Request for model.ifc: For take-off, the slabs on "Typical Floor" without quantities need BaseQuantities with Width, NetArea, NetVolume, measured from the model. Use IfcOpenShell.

First a look at what the model holds.

```python
import ifcopenshell
import ifcopenshell.util.element
import ifcopenshell.util.unit

model = ifcopenshell.open("model.ifc")
print(model.schema)
for unit_type in ("LENGTHUNIT", "AREAUNIT", "VOLUMEUNIT"):
    print(unit_type, ifcopenshell.util.unit.calculate_unit_scale(model, unit_type))
storey = next(s for s in model.by_type("IfcBuildingStorey") if s.Name == "Typical Floor")
slabs = [e for e in ifcopenshell.util.element.get_decomposition(storey) if e.is_a("IfcSlab")]
for e in sorted(slabs, key=lambda e: e.id()):
    print(e.id(), e.is_a(), e.Name, list(ifcopenshell.util.element.get_psets(e, qtos_only=True)), sep=" | ")
```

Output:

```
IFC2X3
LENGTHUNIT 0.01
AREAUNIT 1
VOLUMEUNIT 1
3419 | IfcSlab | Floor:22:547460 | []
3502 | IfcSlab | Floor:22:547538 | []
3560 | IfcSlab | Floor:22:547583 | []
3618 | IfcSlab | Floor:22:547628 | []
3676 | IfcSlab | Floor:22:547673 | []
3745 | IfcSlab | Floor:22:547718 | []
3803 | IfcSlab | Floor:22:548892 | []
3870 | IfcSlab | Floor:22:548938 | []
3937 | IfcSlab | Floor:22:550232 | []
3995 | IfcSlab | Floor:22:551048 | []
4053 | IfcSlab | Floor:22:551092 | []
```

```python
import ifcopenshell
import ifcopenshell.api.pset
import ifcopenshell.geom
import ifcopenshell.util.element
import ifcopenshell.util.shape
import ifcopenshell.util.unit

model = ifcopenshell.open("model.ifc")
unit_scale = ifcopenshell.util.unit.calculate_unit_scale(model)
area_scale = ifcopenshell.util.unit.calculate_unit_scale(model, "AREAUNIT")
volume_scale = ifcopenshell.util.unit.calculate_unit_scale(model, "VOLUMEUNIT")
settings = ifcopenshell.geom.settings()

storey = next(s for s in model.by_type("IfcBuildingStorey") if s.Name == "Typical Floor")
slabs = [e for e in ifcopenshell.util.element.get_decomposition(storey) if e.is_a("IfcSlab")]

for e in sorted(slabs, key=lambda e: e.id()):
    if ifcopenshell.util.element.get_psets(e, qtos_only=True, should_inherit=False):
        continue
    # Geometry comes back in metres, in the element's own axes.
    shape = ifcopenshell.geom.create_shape(settings, e)
    values = {
        "Width": ifcopenshell.util.shape.get_z(shape.geometry) / unit_scale,
        "NetArea": ifcopenshell.util.shape.get_footprint_area(shape.geometry) / area_scale,
        "NetVolume": ifcopenshell.util.shape.get_volume(shape.geometry) / volume_scale,
    }
    qto = ifcopenshell.api.pset.add_qto(model, product=e, name="BaseQuantities")
    ifcopenshell.api.pset.edit_qto(model, qto=qto, properties=values)
    print(e.id(), {k: round(v, 3) for k, v in values.items()})

model.write("model_updated.ifc")
```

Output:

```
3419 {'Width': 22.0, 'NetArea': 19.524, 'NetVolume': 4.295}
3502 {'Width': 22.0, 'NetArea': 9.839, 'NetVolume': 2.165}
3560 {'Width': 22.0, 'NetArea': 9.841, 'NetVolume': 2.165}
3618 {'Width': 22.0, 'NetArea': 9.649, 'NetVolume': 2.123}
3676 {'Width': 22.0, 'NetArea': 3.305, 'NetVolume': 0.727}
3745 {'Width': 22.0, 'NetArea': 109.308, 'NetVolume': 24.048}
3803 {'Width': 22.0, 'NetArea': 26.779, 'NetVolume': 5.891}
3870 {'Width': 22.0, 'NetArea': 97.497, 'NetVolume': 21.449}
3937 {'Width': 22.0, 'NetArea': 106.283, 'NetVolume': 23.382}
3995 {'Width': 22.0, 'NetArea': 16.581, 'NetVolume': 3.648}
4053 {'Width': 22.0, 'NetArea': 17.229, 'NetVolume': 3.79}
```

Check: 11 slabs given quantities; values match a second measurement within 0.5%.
